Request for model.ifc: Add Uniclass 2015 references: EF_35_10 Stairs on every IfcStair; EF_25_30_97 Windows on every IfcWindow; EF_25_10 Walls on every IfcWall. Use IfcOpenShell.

First a look at what the model holds.

```python
import ifcopenshell

model = ifcopenshell.open("model.ifc")
print(model.schema)
print("classifications:", [c.Name for c in model.by_type("IfcClassification")])
for ifc_class in ("IfcDoor", "IfcRoof", "IfcStair", "IfcWall", "IfcWindow"):
    print(ifc_class, len(model.by_type(ifc_class)))
```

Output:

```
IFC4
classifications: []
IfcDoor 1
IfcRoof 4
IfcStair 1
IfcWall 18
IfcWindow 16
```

```python
import ifcopenshell
import ifcopenshell.api.classification

model = ifcopenshell.open("model.ifc")

system = ifcopenshell.api.classification.add_classification(model, classification="Uniclass 2015")

codes = {
    "IfcStair": ("EF_35_10", "Stairs"),
    "IfcWindow": ("EF_25_30_97", "Windows"),
    "IfcWall": ("EF_25_10", "Walls"),
}
for ifc_class, (code, name) in codes.items():
    products = model.by_type(ifc_class)
    ifcopenshell.api.classification.add_reference(
        model, products=products, classification=system, identification=code, name=name
    )
    print(code, len(products))

model.write("model-out.ifc")
```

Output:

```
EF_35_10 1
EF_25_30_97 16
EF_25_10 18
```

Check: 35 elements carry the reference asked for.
